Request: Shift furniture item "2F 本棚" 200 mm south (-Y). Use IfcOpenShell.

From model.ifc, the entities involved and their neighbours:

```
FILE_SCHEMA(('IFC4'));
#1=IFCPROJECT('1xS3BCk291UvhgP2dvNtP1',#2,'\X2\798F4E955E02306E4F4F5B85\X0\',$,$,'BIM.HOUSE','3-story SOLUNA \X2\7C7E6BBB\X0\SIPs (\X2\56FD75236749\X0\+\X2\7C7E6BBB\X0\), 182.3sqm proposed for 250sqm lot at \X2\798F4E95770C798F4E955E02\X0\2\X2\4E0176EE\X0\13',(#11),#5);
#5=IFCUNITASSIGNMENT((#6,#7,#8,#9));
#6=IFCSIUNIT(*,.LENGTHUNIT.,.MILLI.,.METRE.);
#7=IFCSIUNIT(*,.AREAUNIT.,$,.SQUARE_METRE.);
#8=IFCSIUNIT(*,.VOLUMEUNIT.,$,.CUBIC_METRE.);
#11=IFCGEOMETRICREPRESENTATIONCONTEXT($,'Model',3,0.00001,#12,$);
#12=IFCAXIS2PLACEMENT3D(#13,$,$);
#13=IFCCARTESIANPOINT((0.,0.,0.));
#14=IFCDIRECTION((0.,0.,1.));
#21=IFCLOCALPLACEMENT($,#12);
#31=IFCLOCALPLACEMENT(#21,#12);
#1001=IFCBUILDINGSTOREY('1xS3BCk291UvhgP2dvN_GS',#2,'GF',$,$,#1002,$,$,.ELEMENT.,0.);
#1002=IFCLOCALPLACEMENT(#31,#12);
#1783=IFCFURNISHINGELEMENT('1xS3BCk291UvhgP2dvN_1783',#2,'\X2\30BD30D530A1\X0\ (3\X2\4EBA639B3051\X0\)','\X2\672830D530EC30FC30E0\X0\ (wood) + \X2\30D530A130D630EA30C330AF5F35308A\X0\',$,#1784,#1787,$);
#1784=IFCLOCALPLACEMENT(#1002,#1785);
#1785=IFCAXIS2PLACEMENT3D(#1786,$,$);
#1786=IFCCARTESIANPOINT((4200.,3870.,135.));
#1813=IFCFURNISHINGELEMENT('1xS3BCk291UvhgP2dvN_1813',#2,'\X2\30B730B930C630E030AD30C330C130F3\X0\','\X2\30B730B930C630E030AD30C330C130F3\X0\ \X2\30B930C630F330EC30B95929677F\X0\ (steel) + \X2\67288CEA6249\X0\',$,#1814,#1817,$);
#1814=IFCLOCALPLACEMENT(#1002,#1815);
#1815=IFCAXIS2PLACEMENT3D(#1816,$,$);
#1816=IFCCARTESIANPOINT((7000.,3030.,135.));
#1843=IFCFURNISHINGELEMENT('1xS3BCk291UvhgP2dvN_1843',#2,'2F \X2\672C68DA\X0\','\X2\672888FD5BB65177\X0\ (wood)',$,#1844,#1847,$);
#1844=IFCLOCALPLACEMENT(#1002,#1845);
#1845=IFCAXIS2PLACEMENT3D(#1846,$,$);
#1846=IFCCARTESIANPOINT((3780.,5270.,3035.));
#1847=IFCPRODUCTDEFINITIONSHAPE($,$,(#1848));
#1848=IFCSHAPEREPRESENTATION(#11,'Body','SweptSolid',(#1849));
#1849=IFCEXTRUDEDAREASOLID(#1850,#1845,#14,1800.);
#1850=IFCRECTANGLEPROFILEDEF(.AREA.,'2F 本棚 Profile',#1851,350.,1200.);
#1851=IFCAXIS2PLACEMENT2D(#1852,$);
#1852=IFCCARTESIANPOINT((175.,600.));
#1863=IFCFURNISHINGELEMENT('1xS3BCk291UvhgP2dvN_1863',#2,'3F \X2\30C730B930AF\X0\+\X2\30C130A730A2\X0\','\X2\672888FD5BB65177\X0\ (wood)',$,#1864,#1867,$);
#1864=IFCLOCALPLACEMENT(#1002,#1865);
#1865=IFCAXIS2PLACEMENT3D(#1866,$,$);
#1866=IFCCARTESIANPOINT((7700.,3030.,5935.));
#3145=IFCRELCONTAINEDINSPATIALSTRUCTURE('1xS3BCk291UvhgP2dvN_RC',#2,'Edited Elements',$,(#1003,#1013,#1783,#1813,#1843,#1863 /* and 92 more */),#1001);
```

```python
import ifcopenshell
import ifcopenshell.api.geometry
import ifcopenshell.util.placement
import ifcopenshell.util.unit

model = ifcopenshell.open("model.ifc")
unit_scale = ifcopenshell.util.unit.calculate_unit_scale(model)

item = model.by_guid("1xS3BCk291UvhgP2dvN_1843")
matrix = ifcopenshell.util.placement.get_local_placement(item.ObjectPlacement)
matrix[1, 3] -= 0.2 / unit_scale
ifcopenshell.api.geometry.edit_object_placement(model, product=item, matrix=matrix, is_si=False)

print(ifcopenshell.util.placement.get_local_placement(item.ObjectPlacement).round(3) + 0.0)

model.write("model_v2.ifc")
```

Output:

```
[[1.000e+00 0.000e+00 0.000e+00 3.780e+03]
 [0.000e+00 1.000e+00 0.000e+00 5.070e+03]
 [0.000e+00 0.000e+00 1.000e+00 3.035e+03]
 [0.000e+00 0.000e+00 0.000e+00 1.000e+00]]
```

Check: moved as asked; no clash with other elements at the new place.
